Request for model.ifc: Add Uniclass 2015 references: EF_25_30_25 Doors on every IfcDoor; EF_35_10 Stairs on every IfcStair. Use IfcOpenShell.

First a look at what the model holds.

```python
import ifcopenshell

model = ifcopenshell.open("model.ifc")
print(model.schema)
print("classifications:", [c.Name for c in model.by_type("IfcClassification")])
for ifc_class in ("IfcDoor", "IfcRoof", "IfcStair", "IfcWall", "IfcWindow"):
    print(ifc_class, len(model.by_type(ifc_class)))
```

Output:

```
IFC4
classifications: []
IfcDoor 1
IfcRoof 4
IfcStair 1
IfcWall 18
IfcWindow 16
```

```python
import ifcopenshell
import ifcopenshell.api.classification

model = ifcopenshell.open("model.ifc")

system = ifcopenshell.api.classification.add_classification(model, classification="Uniclass 2015")

codes = {
    "IfcDoor": ("EF_25_30_25", "Doors"),
    "IfcStair": ("EF_35_10", "Stairs"),
}
for ifc_class, (code, name) in codes.items():
    products = model.by_type(ifc_class)
    ifcopenshell.api.classification.add_reference(
        model, products=products, classification=system, identification=code, name=name
    )
    print(code, len(products))

model.write("model_v2.ifc")
```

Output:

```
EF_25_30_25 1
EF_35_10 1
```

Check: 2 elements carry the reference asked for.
